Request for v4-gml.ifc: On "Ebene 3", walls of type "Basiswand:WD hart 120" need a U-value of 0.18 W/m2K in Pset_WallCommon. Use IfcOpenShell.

First a look at what the model holds.

```python
import ifcopenshell
import ifcopenshell.util.element

model = ifcopenshell.open("v4-gml.ifc")
print(model.schema)
storey = next(s for s in model.by_type("IfcBuildingStorey") if s.Name == "Ebene 3")
walls = [e for e in ifcopenshell.util.element.get_decomposition(storey) if e.is_a("IfcWall")]
seen = {}
for e in walls:
    element_type = ifcopenshell.util.element.get_type(e)
    key = (element_type.Name if element_type != e and element_type else None, ifcopenshell.util.element.get_pset(e, "Pset_WallCommon", "ThermalTransmittance"))
    seen[key] = seen.get(key, 0) + 1
for (name, value), count in sorted(seen.items(), key=str):
    print(count, "x", name, "|", value)
```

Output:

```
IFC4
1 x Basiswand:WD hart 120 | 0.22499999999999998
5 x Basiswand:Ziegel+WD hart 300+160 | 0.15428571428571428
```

```python
import ifcopenshell
import ifcopenshell.api.pset
import ifcopenshell.util.element

model = ifcopenshell.open("v4-gml.ifc")

storey = next(s for s in model.by_type("IfcBuildingStorey") if s.Name == "Ebene 3")
walls = [e for e in ifcopenshell.util.element.get_decomposition(storey) if e.is_a("IfcWall")]

count = 0
for e in walls:
    element_type = ifcopenshell.util.element.get_type(e)
    if element_type in (None, e) or element_type.Name != "Basiswand:WD hart 120":
        continue
    # add_pset returns the element's existing set when there is one.
    pset = ifcopenshell.api.pset.add_pset(model, product=e, name="Pset_WallCommon")
    ifcopenshell.api.pset.edit_pset(model, pset=pset, properties={"ThermalTransmittance": 0.18})
    count += 1

print(count, "walls updated")

model.write("v4-gml_v2.ifc")
```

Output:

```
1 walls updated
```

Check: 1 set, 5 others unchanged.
